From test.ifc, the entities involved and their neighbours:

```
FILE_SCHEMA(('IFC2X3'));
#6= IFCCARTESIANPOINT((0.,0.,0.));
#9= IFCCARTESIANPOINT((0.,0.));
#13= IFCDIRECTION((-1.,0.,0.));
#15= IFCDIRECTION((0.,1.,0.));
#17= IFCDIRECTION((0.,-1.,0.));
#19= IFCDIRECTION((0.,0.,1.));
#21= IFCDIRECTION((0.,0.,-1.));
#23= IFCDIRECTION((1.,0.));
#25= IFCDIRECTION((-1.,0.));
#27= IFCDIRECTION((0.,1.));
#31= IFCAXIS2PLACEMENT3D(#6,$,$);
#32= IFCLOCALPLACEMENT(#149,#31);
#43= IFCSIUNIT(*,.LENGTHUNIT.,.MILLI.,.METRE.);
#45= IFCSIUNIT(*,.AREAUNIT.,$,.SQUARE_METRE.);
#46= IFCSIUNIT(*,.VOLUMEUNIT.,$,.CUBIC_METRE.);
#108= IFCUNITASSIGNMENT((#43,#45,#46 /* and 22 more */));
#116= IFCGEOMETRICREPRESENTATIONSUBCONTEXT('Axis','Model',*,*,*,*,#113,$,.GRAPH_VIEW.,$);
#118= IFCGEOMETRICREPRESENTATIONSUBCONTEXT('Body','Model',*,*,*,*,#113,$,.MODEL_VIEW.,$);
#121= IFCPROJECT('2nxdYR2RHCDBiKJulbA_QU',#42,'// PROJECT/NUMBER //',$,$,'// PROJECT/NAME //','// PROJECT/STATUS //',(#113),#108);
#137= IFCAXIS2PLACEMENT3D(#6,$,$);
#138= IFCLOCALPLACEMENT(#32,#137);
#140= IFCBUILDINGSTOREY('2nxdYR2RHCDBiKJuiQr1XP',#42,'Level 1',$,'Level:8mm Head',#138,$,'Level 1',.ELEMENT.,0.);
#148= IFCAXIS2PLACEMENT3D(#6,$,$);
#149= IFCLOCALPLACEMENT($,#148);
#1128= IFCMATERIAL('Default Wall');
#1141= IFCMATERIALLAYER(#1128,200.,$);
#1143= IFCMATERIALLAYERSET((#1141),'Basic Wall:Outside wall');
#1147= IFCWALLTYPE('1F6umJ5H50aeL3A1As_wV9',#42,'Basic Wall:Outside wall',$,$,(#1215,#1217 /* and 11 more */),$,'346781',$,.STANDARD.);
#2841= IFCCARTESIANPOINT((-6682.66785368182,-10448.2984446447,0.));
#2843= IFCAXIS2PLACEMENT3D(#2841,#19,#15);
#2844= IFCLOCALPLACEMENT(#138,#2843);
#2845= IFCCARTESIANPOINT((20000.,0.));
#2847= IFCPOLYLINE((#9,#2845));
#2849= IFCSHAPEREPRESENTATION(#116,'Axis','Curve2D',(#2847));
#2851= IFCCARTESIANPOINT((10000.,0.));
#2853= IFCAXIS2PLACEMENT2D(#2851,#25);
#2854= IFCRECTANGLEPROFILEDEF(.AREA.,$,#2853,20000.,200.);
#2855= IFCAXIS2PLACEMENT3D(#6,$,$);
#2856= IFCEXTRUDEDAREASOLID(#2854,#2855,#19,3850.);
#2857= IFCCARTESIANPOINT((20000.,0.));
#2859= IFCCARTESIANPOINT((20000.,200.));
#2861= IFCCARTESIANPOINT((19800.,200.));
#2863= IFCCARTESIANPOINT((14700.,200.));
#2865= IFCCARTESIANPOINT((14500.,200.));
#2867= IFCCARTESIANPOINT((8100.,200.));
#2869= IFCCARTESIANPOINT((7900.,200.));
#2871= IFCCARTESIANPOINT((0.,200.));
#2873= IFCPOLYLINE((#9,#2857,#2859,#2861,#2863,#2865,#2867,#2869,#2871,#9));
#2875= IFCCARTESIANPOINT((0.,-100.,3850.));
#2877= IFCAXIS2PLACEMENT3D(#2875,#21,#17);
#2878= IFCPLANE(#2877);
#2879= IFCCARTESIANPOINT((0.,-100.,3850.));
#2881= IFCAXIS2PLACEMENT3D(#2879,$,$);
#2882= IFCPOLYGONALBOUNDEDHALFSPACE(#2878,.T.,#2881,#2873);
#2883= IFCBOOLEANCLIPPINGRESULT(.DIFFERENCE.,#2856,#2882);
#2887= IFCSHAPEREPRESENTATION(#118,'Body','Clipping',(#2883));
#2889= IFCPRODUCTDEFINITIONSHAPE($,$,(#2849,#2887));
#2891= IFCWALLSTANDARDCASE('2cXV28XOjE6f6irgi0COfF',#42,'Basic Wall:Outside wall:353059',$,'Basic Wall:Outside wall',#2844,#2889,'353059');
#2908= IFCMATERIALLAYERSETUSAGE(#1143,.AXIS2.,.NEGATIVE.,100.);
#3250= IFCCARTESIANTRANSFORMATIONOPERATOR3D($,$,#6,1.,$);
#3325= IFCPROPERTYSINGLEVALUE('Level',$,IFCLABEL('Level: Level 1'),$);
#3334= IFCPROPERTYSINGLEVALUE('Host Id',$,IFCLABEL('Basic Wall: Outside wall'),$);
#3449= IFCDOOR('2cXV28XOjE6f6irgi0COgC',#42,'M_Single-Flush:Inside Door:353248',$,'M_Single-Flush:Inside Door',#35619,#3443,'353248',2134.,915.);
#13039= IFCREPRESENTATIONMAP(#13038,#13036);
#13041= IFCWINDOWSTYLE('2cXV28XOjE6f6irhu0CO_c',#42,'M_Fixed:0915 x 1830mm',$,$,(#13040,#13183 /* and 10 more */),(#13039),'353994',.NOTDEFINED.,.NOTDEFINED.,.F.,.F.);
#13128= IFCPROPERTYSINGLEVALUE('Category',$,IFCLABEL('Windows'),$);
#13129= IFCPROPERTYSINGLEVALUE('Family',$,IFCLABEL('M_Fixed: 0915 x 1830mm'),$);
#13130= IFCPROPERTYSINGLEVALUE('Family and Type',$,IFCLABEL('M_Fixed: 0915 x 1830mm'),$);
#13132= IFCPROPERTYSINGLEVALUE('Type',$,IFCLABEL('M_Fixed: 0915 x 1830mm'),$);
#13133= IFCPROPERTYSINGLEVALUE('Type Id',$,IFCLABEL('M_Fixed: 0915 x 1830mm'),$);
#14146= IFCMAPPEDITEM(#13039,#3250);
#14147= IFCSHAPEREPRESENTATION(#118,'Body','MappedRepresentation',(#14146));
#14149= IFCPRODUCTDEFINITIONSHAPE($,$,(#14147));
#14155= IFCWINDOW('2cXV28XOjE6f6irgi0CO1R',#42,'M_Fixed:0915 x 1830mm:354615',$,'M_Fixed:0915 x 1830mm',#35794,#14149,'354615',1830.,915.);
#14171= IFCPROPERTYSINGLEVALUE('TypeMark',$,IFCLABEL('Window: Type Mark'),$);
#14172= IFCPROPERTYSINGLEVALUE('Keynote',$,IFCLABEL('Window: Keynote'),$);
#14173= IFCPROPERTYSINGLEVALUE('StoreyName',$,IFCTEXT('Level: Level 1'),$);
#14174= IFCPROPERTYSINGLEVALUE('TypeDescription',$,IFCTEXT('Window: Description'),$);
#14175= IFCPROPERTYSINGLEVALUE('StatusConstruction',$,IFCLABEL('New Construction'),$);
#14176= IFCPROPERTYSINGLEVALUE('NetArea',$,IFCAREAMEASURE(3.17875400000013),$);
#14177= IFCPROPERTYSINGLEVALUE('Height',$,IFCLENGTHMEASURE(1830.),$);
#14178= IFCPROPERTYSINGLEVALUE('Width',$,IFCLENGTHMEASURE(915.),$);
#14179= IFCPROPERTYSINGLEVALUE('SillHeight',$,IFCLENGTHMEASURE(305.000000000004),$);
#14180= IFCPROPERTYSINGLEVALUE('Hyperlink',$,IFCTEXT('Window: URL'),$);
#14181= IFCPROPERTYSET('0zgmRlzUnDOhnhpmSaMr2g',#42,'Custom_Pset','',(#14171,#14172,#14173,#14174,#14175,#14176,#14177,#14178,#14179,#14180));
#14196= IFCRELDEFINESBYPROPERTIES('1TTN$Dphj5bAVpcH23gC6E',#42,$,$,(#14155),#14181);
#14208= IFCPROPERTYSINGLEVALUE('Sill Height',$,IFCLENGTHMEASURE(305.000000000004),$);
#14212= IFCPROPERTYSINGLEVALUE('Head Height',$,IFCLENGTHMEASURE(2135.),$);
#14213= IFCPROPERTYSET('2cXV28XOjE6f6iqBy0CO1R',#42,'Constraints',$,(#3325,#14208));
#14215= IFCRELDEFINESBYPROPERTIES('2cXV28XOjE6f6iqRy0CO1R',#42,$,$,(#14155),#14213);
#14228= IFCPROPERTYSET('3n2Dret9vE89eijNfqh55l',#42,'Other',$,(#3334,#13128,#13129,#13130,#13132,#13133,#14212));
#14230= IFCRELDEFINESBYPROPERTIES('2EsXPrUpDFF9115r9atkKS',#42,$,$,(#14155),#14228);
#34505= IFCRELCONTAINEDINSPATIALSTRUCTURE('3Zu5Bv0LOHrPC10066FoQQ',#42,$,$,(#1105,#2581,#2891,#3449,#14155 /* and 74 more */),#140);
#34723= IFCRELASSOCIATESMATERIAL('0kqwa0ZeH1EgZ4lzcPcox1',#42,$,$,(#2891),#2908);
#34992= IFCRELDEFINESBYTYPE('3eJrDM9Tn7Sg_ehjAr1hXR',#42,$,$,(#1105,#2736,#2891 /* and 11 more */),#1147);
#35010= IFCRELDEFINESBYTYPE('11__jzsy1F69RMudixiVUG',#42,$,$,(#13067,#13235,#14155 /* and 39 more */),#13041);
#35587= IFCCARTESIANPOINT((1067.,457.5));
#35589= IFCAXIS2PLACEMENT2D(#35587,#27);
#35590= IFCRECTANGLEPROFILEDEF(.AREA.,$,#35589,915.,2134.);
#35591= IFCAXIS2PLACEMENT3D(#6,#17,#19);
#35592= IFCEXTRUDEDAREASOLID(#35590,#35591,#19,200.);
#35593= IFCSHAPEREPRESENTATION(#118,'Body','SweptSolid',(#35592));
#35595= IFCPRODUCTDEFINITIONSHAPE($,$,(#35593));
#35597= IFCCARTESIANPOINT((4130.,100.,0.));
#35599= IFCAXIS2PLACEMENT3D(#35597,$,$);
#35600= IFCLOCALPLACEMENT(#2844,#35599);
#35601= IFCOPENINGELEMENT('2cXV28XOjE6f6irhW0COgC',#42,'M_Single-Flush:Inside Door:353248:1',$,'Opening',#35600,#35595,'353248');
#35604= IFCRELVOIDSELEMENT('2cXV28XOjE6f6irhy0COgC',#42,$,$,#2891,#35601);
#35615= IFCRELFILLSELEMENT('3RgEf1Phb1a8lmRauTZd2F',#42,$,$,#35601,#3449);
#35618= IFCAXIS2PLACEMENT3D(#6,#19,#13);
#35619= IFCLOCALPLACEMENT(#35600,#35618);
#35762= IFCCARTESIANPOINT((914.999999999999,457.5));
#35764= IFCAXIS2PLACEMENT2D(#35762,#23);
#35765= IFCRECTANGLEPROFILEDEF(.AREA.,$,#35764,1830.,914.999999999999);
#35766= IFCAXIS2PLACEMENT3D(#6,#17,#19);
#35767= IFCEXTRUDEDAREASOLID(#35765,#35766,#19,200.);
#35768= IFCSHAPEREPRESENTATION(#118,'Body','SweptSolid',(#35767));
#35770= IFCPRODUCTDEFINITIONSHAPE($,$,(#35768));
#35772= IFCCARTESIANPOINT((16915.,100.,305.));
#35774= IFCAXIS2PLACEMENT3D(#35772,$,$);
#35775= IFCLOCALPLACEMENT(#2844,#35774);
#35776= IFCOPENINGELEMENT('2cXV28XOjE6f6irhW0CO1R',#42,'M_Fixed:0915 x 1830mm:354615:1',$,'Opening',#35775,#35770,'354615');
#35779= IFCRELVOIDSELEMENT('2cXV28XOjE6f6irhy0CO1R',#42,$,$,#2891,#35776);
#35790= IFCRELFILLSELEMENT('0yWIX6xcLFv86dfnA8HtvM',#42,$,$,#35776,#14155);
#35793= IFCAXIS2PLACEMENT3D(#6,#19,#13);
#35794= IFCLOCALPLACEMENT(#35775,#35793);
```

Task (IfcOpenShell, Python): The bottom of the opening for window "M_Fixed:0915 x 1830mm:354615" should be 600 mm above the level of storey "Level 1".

```python
import numpy as np
import ifcopenshell
import ifcopenshell.api.geometry
import ifcopenshell.api.pset
import ifcopenshell.geom
import ifcopenshell.util.element
import ifcopenshell.util.placement
import ifcopenshell.util.shape
import ifcopenshell.util.unit

model = ifcopenshell.open("test.ifc")
unit_scale = ifcopenshell.util.unit.calculate_unit_scale(model)

window = model.by_id(14155)
opening = window.FillsVoids[0].RelatingOpeningElement
storey = ifcopenshell.util.element.get_container(window, ifc_class="IfcBuildingStorey")
level = ifcopenshell.util.placement.get_local_placement(storey.ObjectPlacement)[2, 3]

# The opening's origin need not be at the sill, so measure its lowest point.
shape = ifcopenshell.geom.create_shape(ifcopenshell.geom.settings(), opening)
bottom = ifcopenshell.util.shape.get_shape_bottom_elevation(shape, shape.geometry) / unit_scale
dz = level + 600.0 - bottom

shift = np.array([0.0, 0.0, dz])
# The window is placed relative to its opening, so it follows when the opening moves.
matrix = ifcopenshell.util.placement.get_local_placement(opening.ObjectPlacement)
matrix[:3, 3] += shift
ifcopenshell.api.geometry.edit_object_placement(
    model, product=opening, matrix=matrix, is_si=False, should_transform_children=True
)

# Keep the stored heights in step.
pset = model.by_id(ifcopenshell.util.element.get_pset(window, "Custom_Pset", should_inherit=False)["id"])
ifcopenshell.api.pset.edit_pset(model, pset=pset, properties={
    "SillHeight": model.create_entity("IfcLengthMeasure", ifcopenshell.util.element.get_pset(window, "Constraints", "Sill Height") + dz),
})
pset = model.by_id(ifcopenshell.util.element.get_pset(window, "Constraints", should_inherit=False)["id"])
ifcopenshell.api.pset.edit_pset(model, pset=pset, properties={
    "Sill Height": model.create_entity("IfcLengthMeasure", ifcopenshell.util.element.get_pset(window, "Constraints", "Sill Height") + dz),
})
pset = model.by_id(ifcopenshell.util.element.get_pset(window, "Other", should_inherit=False)["id"])
ifcopenshell.api.pset.edit_pset(model, pset=pset, properties={
    "Head Height": model.create_entity("IfcLengthMeasure", ifcopenshell.util.element.get_pset(window, "Other", "Head Height") + dz),
})

print(f"moved by {dz * unit_scale:+.3f} m")

model.write("test_v2.ifc")
```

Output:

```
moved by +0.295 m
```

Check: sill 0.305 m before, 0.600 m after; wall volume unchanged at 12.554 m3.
